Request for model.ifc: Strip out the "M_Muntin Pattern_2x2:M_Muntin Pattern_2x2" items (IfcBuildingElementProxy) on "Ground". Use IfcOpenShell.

First a look at what the model holds.

```python
import ifcopenshell
import ifcopenshell.util.element

model = ifcopenshell.open("model.ifc")
print(model.schema)
storey = next(s for s in model.by_type("IfcBuildingStorey") if s.Name == "Ground")
proxies = [e for e in ifcopenshell.util.element.get_decomposition(storey) if e.is_a("IfcBuildingElementProxy")]
seen = {}
for e in proxies:
    element_type = ifcopenshell.util.element.get_type(e)
    name = element_type.Name if element_type not in (None, e) else None
    seen[name] = seen.get(name, 0) + 1
for name, count in sorted(seen.items(), key=str):
    print(count, "x", name)
```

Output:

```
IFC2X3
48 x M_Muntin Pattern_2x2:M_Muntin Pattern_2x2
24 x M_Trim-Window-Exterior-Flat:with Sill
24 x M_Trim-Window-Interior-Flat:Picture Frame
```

```python
import ifcopenshell
import ifcopenshell.api.root
import ifcopenshell.util.element

model = ifcopenshell.open("model.ifc")

storey = next(s for s in model.by_type("IfcBuildingStorey") if s.Name == "Ground")
proxies = [e for e in ifcopenshell.util.element.get_decomposition(storey) if e.is_a("IfcBuildingElementProxy")]
targets = [e for e in proxies if (t := ifcopenshell.util.element.get_type(e)) not in (None, e) and t.Name == "M_Muntin Pattern_2x2:M_Muntin Pattern_2x2"]

for e in targets:
    ifcopenshell.api.root.remove_product(model, product=e)
print(len(targets), "removed")

model.write("model_rev.ifc")
```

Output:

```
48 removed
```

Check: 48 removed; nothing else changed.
